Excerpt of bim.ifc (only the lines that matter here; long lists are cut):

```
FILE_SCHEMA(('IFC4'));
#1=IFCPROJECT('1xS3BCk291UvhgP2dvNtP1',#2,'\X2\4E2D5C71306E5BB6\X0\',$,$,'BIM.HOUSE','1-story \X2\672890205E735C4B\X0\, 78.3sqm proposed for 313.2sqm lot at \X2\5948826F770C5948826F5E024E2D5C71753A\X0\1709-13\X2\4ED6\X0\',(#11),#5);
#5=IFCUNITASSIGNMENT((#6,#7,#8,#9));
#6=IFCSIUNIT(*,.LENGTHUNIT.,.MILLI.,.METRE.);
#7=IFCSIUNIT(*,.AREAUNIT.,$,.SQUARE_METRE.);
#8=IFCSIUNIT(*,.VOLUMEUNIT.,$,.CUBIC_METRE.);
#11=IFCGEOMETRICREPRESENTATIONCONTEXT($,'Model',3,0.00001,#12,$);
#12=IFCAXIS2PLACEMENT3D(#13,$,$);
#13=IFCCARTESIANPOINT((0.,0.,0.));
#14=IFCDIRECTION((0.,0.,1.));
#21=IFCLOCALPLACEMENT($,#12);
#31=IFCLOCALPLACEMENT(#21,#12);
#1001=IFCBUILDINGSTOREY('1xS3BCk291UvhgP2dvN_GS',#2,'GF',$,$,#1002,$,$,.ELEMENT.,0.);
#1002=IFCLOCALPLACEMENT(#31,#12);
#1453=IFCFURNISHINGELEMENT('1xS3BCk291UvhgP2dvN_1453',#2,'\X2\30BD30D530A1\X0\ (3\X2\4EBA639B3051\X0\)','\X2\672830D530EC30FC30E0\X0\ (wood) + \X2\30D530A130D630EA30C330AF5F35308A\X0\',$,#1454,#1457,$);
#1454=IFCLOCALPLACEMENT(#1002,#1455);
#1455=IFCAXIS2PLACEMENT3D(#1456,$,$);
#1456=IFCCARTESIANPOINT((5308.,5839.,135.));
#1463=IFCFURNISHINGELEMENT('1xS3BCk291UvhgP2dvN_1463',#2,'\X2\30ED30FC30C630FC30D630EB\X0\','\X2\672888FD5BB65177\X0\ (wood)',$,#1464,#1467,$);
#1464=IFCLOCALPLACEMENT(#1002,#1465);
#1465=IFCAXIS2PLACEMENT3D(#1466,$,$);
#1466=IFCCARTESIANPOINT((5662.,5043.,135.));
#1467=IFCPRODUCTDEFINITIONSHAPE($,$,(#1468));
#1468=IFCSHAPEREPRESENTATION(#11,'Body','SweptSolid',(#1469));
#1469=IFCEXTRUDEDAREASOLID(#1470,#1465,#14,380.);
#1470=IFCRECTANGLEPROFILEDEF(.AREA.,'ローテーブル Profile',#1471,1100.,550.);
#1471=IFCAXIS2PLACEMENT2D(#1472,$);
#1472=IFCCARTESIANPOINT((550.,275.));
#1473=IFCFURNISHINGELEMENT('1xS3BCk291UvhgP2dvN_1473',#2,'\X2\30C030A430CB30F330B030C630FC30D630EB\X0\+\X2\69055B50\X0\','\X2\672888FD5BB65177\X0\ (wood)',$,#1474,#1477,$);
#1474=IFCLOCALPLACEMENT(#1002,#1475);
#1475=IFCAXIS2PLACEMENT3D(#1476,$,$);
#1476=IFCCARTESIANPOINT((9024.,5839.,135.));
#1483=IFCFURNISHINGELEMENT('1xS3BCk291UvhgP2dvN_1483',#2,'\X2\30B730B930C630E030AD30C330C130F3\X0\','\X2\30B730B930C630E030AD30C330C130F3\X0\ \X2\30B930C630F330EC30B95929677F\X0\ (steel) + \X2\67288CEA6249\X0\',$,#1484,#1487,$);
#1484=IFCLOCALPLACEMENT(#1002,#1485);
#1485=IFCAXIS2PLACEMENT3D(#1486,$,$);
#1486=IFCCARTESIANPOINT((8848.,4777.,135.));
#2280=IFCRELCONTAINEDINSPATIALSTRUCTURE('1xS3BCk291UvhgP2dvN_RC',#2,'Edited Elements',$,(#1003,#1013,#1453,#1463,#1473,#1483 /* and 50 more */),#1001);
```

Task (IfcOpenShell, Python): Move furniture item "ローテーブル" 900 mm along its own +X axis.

```python
import ifcopenshell
import ifcopenshell.api.geometry
import ifcopenshell.util.placement

model = ifcopenshell.open("bim.ifc")

item = model.by_id(1463)
matrix = ifcopenshell.util.placement.get_local_placement(item.ObjectPlacement)
matrix[:3, 3] += matrix[:3, 0] * 900.0
ifcopenshell.api.geometry.edit_object_placement(model, product=item, matrix=matrix, is_si=False)

print(ifcopenshell.util.placement.get_local_placement(item.ObjectPlacement).round(3) + 0.0)

model.write("bim-out.ifc")
```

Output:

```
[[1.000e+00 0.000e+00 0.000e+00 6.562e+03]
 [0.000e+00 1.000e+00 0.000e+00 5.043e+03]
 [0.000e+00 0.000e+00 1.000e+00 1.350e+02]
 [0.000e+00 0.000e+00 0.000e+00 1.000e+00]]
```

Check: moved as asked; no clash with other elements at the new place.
